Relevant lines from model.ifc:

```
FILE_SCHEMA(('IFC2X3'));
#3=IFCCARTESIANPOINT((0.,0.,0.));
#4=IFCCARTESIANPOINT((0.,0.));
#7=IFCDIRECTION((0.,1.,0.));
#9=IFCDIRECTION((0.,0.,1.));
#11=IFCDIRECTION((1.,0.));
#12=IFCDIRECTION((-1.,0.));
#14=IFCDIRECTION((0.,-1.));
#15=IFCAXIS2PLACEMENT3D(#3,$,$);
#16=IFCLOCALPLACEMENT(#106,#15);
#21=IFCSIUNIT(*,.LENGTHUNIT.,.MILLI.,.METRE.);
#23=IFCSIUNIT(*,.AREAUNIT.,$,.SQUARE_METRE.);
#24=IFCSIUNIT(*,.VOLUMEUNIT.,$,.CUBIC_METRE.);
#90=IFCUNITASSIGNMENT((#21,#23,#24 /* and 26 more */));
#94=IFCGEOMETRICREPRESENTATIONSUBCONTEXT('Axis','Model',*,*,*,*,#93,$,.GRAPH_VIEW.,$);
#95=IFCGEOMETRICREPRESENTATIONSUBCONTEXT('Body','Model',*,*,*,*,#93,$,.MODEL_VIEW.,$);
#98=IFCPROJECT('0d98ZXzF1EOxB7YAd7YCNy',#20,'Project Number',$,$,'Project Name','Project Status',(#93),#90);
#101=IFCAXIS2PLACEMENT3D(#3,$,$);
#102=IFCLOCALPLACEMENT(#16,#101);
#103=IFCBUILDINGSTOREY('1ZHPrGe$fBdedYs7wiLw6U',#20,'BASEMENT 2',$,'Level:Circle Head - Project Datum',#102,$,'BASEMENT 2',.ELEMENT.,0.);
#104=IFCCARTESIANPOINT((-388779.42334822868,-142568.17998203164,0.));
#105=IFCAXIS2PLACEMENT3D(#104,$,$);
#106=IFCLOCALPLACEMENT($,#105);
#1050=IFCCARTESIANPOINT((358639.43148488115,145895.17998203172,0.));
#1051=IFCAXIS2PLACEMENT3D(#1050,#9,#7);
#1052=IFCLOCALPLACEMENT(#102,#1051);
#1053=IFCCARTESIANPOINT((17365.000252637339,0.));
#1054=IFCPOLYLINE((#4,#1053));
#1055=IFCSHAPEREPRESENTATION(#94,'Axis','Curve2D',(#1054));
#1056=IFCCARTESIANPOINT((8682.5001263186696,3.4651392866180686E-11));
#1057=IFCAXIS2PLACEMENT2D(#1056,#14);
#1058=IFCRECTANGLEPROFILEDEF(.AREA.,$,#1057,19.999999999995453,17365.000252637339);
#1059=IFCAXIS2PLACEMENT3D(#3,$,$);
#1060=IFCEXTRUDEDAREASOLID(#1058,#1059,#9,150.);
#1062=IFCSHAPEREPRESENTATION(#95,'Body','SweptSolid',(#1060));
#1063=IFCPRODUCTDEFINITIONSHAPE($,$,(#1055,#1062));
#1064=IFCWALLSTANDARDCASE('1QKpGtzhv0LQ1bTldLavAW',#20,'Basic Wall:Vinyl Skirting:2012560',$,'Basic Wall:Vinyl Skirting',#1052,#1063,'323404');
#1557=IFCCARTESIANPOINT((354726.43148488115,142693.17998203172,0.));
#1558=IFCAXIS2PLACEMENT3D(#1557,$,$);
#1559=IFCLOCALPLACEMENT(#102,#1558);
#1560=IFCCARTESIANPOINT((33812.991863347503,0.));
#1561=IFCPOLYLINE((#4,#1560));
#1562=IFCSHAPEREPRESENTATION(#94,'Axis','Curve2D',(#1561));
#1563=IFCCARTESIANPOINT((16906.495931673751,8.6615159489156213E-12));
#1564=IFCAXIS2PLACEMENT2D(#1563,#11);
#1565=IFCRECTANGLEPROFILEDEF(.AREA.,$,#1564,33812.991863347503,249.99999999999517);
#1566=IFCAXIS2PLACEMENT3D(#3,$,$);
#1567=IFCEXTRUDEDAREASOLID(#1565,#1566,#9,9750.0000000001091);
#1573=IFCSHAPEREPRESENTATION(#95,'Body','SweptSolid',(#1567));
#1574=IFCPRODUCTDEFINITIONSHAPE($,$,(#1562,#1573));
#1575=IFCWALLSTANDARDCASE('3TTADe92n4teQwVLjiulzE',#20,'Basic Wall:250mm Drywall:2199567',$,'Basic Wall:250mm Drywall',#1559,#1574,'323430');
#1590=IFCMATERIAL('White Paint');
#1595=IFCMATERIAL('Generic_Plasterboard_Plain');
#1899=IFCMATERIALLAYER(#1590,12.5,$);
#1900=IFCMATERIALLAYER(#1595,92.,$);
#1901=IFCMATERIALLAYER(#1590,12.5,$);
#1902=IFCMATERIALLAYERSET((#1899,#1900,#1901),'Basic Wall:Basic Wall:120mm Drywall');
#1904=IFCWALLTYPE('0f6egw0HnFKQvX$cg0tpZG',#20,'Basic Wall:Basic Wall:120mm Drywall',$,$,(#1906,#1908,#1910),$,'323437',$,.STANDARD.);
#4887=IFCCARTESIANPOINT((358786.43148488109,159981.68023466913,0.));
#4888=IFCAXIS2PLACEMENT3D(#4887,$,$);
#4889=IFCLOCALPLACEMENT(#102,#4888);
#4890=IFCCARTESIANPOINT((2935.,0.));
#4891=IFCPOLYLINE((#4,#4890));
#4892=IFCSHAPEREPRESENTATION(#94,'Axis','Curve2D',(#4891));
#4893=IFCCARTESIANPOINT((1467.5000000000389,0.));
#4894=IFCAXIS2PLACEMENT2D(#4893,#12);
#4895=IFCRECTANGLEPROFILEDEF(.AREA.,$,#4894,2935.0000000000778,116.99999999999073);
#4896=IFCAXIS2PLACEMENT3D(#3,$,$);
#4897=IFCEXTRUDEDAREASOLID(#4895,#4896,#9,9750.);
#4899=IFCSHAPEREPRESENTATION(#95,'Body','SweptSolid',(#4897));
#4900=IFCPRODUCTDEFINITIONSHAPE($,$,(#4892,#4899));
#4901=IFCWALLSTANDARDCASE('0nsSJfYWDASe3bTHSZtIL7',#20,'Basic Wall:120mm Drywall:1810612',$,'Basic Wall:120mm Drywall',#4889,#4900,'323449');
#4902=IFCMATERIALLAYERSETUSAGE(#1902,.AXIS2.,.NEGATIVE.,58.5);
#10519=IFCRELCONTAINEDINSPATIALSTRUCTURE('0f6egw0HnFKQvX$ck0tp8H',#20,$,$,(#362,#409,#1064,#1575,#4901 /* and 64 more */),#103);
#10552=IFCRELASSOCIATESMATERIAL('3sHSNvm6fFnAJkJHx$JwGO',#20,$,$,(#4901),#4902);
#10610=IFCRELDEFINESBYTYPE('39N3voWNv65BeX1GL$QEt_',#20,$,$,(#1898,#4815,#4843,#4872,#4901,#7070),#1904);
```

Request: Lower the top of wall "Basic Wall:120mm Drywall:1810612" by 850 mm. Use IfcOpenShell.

```python
import ifcopenshell
import ifcopenshell.geom
import ifcopenshell.util.representation
import ifcopenshell.util.shape

model = ifcopenshell.open("model.ifc")
settings = ifcopenshell.geom.settings()


def volume(element):
    """Net volume in cubic metres, openings subtracted."""
    shape = ifcopenshell.geom.create_shape(settings, element)
    return ifcopenshell.util.shape.get_volume(shape.geometry)


wall = model.by_id(4901)
before = volume(wall)

body = ifcopenshell.util.representation.get_representation(wall, "Model", "Body")
solid = body.Items[0]
old_height = solid.Depth
solid.Depth -= 850.0
after = volume(wall)

print(f"height {old_height:g} -> {solid.Depth:g}, volume {before:.3f} -> {after:.3f} m3")

model.write("model_updated.ifc")
```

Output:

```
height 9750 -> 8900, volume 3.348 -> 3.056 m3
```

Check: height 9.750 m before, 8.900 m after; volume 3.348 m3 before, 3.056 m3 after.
